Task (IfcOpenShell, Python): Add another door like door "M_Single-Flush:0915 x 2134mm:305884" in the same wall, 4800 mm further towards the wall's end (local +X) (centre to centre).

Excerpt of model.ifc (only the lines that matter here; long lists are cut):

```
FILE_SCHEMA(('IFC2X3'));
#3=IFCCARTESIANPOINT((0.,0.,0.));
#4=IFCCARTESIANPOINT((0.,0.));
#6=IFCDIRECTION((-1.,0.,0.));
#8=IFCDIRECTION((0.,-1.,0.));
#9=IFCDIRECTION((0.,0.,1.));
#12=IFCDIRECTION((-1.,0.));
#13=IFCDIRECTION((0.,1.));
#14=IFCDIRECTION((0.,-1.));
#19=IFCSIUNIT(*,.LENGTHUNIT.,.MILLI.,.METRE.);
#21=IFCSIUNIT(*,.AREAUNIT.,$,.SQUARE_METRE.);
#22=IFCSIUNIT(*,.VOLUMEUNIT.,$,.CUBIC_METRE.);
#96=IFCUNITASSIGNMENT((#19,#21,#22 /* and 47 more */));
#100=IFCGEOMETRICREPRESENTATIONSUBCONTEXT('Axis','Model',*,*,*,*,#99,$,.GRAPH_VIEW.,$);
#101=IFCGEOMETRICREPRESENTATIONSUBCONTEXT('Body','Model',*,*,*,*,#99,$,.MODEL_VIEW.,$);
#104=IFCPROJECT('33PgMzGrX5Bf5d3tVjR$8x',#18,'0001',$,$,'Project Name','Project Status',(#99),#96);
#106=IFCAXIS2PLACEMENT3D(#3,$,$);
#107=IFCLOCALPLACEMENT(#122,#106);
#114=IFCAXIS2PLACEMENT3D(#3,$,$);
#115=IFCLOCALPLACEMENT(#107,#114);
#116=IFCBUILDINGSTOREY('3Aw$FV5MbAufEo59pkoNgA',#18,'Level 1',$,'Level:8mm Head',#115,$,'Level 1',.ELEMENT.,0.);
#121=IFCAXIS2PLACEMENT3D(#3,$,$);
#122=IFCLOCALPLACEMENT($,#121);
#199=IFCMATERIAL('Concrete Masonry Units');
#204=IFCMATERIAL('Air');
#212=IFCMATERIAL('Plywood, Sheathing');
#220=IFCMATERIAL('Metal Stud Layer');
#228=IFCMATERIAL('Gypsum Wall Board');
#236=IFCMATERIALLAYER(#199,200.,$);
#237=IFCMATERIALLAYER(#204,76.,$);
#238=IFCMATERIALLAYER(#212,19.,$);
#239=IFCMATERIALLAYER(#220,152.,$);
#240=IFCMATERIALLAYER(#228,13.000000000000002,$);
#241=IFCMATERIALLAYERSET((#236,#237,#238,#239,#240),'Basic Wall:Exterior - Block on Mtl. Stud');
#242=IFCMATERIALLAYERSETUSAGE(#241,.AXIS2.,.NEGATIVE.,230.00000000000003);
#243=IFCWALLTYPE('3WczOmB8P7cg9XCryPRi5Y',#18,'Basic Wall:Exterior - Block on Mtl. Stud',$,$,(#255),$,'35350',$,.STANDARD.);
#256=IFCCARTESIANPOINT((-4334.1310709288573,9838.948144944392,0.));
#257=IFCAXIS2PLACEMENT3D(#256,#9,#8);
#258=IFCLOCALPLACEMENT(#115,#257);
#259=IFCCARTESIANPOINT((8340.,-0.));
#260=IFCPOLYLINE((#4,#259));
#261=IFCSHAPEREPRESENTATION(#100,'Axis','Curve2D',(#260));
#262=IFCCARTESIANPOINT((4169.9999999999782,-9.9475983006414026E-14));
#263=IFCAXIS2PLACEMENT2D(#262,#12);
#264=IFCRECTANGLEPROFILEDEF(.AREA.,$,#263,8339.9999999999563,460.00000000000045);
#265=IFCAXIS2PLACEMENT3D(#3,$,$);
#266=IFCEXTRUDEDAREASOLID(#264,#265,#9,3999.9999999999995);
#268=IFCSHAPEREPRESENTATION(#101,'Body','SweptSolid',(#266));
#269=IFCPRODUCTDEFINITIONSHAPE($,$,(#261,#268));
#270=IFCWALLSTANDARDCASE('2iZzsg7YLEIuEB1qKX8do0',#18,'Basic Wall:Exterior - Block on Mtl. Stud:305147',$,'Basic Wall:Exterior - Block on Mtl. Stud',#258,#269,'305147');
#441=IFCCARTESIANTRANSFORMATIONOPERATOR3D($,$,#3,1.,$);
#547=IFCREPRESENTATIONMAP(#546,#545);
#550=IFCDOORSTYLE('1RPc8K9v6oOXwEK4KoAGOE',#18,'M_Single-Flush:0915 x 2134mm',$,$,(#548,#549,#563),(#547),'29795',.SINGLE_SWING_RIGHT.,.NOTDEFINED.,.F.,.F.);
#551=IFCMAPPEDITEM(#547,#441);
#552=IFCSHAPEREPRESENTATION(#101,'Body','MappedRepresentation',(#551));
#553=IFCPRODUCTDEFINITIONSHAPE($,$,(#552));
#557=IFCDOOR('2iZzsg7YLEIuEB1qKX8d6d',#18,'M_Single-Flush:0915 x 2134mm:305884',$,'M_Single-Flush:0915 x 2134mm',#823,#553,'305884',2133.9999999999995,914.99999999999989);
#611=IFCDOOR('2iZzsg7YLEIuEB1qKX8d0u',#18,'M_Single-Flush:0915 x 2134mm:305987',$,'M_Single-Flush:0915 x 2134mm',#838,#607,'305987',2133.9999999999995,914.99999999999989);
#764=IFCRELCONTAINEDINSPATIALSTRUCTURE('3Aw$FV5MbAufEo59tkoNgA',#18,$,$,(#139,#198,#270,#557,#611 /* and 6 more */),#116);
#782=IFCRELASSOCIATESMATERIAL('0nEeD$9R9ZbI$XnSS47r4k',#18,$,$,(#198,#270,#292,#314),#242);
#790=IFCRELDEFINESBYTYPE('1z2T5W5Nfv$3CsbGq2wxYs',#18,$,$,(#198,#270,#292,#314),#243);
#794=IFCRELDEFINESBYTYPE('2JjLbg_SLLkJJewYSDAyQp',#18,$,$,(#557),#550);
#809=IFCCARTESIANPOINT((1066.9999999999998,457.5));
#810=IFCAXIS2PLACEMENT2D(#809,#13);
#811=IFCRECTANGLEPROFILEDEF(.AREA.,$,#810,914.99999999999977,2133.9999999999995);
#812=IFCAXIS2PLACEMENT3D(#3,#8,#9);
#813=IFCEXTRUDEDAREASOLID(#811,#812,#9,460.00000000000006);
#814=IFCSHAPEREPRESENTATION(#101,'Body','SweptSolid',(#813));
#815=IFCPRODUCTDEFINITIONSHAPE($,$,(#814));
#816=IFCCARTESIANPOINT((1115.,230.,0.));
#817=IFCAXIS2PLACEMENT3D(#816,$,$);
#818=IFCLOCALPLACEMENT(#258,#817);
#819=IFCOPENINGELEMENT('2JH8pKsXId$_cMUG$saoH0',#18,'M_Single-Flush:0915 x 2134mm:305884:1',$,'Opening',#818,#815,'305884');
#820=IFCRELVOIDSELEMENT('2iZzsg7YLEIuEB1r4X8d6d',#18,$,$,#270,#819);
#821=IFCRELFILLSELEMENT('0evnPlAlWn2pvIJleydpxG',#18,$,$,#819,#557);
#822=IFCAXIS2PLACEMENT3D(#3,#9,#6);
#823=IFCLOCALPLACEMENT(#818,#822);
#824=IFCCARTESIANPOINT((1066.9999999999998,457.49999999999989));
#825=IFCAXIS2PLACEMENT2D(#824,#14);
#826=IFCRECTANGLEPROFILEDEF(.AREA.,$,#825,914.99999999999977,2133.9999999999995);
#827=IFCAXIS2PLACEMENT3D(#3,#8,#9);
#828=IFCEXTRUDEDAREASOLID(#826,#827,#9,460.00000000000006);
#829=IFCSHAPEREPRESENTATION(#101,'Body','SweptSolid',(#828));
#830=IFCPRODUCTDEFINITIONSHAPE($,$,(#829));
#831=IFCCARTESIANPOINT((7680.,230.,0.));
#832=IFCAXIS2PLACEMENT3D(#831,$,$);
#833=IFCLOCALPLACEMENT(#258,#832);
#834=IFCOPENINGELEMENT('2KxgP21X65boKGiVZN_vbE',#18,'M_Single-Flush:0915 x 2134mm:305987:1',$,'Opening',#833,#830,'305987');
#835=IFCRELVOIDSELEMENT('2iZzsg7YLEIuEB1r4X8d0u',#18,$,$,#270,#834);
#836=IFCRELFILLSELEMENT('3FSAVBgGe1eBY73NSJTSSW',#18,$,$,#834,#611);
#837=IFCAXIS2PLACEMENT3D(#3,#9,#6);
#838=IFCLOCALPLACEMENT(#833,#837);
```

```python
import ifcopenshell
import ifcopenshell.api.feature
import ifcopenshell.api.geometry
import ifcopenshell.api.root
import ifcopenshell.geom
import ifcopenshell.util.element
import ifcopenshell.util.placement
import ifcopenshell.util.shape

model = ifcopenshell.open("model.ifc")
settings = ifcopenshell.geom.settings()


def volume(element):
    """Net volume in cubic metres, openings subtracted."""
    shape = ifcopenshell.geom.create_shape(settings, element)
    return ifcopenshell.util.shape.get_volume(shape.geometry)


def reuse_history(source, copy):
    """copy_class also copies each property set's owner history, people and application; keep the originals."""
    for rel in copy.IsDefinedBy:
        if rel.is_a("IfcRelDefinesByProperties") and (history := rel.RelatingPropertyDefinition.OwnerHistory):
            rel.RelatingPropertyDefinition.OwnerHistory = source.OwnerHistory
            ifcopenshell.util.element.remove_deep2(model, history)


door = model.by_id(557)
opening = door.FillsVoids[0].RelatingOpeningElement
wall = opening.VoidsElements[0].RelatingBuildingElement
before = volume(wall)
shift = ifcopenshell.util.placement.get_local_placement(wall.ObjectPlacement)[:3, 0] * 4800.0

# copy_class copies the void relationship, type, container and properties, but no geometry.
new_opening = ifcopenshell.api.root.copy_class(model, product=opening)
new_opening.Representation = ifcopenshell.util.element.copy_deep(
    model, opening.Representation, exclude=["IfcGeometricRepresentationContext", "IfcRepresentationMap"]
)
new_opening.Name = "M_Single-Flush:0915 x 2134mm"
new_opening.Tag = None
new_door = ifcopenshell.api.root.copy_class(model, product=door)
new_door.Representation = ifcopenshell.util.element.copy_deep(
    model, door.Representation, exclude=["IfcGeometricRepresentationContext", "IfcRepresentationMap"]
)
new_door.Name = "M_Single-Flush:0915 x 2134mm"
new_door.Tag = None
reuse_history(door, new_door)
fills = ifcopenshell.api.feature.add_filling(model, opening=new_opening, element=new_door)
fills.OwnerHistory = new_door.OwnerHistory  # required in IFC2X3

for old, new in ((opening, new_opening), (door, new_door)):
    matrix = ifcopenshell.util.placement.get_local_placement(old.ObjectPlacement)
    matrix[:3, 3] += shift
    ifcopenshell.api.geometry.edit_object_placement(model, product=new, matrix=matrix, is_si=False)

after = volume(wall)

print(f"wall volume {before:.3f} -> {after:.3f} m3")

model.write("model_v2.ifc")
```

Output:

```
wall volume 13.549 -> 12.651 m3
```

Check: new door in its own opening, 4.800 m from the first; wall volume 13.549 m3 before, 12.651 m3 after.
